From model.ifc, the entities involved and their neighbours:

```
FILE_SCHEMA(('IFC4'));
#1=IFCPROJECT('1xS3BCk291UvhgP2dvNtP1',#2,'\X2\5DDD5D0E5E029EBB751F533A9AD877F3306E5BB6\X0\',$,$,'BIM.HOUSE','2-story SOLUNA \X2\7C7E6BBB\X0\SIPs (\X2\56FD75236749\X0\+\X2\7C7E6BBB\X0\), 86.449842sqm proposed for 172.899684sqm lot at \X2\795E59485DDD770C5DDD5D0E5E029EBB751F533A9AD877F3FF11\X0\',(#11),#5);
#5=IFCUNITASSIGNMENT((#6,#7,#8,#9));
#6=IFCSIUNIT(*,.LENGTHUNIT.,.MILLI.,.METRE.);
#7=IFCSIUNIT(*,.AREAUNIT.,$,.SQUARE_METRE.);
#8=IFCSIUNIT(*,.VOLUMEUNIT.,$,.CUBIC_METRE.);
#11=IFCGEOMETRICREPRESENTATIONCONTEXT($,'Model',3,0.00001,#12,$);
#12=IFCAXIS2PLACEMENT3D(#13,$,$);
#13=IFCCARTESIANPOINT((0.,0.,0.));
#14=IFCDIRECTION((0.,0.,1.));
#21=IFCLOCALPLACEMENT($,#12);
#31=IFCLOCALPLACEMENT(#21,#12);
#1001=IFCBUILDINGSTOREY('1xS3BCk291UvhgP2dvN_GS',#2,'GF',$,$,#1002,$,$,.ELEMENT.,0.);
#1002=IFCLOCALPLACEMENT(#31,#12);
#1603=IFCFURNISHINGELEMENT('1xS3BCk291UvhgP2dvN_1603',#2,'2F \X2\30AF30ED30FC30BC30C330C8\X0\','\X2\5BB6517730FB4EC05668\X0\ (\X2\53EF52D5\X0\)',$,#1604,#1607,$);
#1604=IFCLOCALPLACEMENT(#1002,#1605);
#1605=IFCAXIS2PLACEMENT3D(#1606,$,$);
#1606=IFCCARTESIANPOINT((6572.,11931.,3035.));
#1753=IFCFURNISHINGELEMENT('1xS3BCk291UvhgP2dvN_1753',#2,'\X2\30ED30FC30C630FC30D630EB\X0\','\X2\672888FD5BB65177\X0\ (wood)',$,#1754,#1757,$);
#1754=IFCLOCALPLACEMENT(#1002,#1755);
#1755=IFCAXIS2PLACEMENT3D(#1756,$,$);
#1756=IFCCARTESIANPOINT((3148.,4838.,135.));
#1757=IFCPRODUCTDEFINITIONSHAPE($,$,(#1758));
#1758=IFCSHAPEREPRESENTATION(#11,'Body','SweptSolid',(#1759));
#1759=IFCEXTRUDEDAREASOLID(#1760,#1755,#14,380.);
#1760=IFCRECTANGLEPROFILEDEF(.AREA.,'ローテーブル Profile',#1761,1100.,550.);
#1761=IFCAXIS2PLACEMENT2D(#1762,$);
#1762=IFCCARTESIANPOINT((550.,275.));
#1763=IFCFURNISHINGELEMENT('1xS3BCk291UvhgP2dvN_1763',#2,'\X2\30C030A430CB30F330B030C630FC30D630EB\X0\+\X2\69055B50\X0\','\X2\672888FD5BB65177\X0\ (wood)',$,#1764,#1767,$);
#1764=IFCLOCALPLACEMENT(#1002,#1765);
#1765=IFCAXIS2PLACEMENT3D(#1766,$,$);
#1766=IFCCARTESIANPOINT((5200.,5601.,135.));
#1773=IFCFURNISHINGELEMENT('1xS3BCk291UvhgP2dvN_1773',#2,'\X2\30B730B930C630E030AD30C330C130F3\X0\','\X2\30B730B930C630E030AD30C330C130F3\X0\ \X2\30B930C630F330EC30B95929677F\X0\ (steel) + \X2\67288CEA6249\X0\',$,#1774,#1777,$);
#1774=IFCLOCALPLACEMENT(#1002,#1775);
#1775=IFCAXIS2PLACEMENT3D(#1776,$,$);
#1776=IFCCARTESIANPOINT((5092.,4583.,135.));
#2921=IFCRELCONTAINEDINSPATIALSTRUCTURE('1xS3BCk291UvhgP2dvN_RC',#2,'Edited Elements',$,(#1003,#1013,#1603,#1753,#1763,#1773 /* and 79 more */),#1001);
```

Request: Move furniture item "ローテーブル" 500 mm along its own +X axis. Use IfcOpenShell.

```python
import ifcopenshell
import ifcopenshell.api.geometry
import ifcopenshell.util.placement

model = ifcopenshell.open("model.ifc")

item = model.by_guid("1xS3BCk291UvhgP2dvN_1753")
matrix = ifcopenshell.util.placement.get_local_placement(item.ObjectPlacement)
matrix[:3, 3] += matrix[:3, 0] * 500.0
ifcopenshell.api.geometry.edit_object_placement(model, product=item, matrix=matrix, is_si=False)

print(ifcopenshell.util.placement.get_local_placement(item.ObjectPlacement).round(3) + 0.0)

model.write("model_updated.ifc")
```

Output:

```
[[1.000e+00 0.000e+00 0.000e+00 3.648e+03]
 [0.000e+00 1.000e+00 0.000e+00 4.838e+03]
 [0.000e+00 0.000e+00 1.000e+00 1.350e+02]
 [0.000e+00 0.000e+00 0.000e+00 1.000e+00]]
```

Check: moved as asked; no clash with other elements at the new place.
